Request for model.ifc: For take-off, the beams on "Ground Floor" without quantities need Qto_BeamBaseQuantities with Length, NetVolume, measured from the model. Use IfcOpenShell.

First a look at what the model holds.

```python
import ifcopenshell
import ifcopenshell.util.element
import ifcopenshell.util.unit

model = ifcopenshell.open("model.ifc")
print(model.schema)
for unit_type in ("LENGTHUNIT", "AREAUNIT", "VOLUMEUNIT"):
    print(unit_type, ifcopenshell.util.unit.calculate_unit_scale(model, unit_type))
storey = next(s for s in model.by_type("IfcBuildingStorey") if s.Name == "Ground Floor")
beams = [e for e in ifcopenshell.util.element.get_decomposition(storey) if e.is_a("IfcBeam")]
for e in sorted(beams, key=lambda e: e.id()):
    print(e.id(), e.is_a(), e.Name, list(ifcopenshell.util.element.get_psets(e, qtos_only=True)), sep=" | ")
```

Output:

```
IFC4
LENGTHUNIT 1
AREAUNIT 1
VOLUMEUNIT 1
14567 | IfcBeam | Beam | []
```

```python
import ifcopenshell
import ifcopenshell.api.pset
import ifcopenshell.geom
import ifcopenshell.util.element
import ifcopenshell.util.shape
import ifcopenshell.util.unit

model = ifcopenshell.open("model.ifc")
unit_scale = ifcopenshell.util.unit.calculate_unit_scale(model)
volume_scale = ifcopenshell.util.unit.calculate_unit_scale(model, "VOLUMEUNIT")
settings = ifcopenshell.geom.settings()

storey = next(s for s in model.by_type("IfcBuildingStorey") if s.Name == "Ground Floor")
beams = [e for e in ifcopenshell.util.element.get_decomposition(storey) if e.is_a("IfcBeam")]

for e in sorted(beams, key=lambda e: e.id()):
    if ifcopenshell.util.element.get_psets(e, qtos_only=True, should_inherit=False):
        continue
    # Geometry comes back in metres, in the element's own axes.
    shape = ifcopenshell.geom.create_shape(settings, e)
    values = {
        "Length": ifcopenshell.util.shape.get_max_xyz(shape.geometry) / unit_scale,
        "NetVolume": ifcopenshell.util.shape.get_volume(shape.geometry) / volume_scale,
    }
    qto = ifcopenshell.api.pset.add_qto(model, product=e, name="Qto_BeamBaseQuantities")
    ifcopenshell.api.pset.edit_qto(model, qto=qto, properties=values)
    print(e.id(), {k: round(v, 3) for k, v in values.items()})

model.write("model-out.ifc")
```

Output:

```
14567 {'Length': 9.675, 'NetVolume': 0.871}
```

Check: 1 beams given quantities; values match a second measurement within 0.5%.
